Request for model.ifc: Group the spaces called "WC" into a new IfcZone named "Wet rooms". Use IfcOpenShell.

First a look at what the model holds.

```python
import ifcopenshell

model = ifcopenshell.open("model.ifc")
print(model.schema)
seen = {}
for space in model.by_type("IfcSpace"):
    seen[space.LongName] = seen.get(space.LongName, 0) + 1
for name, count in sorted(seen.items(), key=str):
    print(count, "x", name)
print("zones:", [z.Name for z in model.by_type("IfcZone")][:20])
```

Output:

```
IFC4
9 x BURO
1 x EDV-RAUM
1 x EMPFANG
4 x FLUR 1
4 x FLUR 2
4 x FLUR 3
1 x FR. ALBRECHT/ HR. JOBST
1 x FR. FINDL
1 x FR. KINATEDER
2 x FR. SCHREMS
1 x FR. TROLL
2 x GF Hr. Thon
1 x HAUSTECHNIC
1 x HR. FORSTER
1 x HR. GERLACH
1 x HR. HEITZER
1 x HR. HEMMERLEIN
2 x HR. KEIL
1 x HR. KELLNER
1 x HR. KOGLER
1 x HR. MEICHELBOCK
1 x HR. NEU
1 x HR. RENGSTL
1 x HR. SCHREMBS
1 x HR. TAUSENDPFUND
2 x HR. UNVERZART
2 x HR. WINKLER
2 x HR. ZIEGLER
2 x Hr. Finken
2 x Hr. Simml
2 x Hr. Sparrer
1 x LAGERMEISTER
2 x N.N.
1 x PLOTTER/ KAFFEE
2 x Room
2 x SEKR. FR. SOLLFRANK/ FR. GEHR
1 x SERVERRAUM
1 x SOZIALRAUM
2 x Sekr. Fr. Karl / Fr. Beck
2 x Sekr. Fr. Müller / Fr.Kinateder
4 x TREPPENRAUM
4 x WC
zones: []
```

```python
import ifcopenshell
import ifcopenshell.api.group
import ifcopenshell.api.root

model = ifcopenshell.open("model.ifc")

names = {"WC"}
spaces = [s for s in model.by_type("IfcSpace") if s.LongName in names]

zone = ifcopenshell.api.root.create_entity(model, ifc_class="IfcZone", name="Wet rooms")
ifcopenshell.api.group.assign_group(model, products=spaces, group=zone)
print(len(spaces), "spaces in", zone.Name)

model.write("model_edited.ifc")
```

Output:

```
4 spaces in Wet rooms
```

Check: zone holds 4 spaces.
